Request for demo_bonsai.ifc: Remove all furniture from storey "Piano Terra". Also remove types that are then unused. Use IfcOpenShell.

First a look at what the model holds.

```python
import ifcopenshell
import ifcopenshell.util.element

model = ifcopenshell.open("demo_bonsai.ifc")
print(model.schema)
storey = next(s for s in model.by_type("IfcBuildingStorey") if s.Name == "Piano Terra")
furniture = [e for e in ifcopenshell.util.element.get_decomposition(storey) if e.is_a("IfcFurnishingElement")]
seen = {}
for e in furniture:
    element_type = ifcopenshell.util.element.get_type(e)
    name = element_type.Name if element_type not in (None, e) else None
    seen[name] = seen.get(name, 0) + 1
for name, count in sorted(seen.items(), key=str):
    print(count, "x", name)
```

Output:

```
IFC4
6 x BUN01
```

```python
import ifcopenshell
import ifcopenshell.api.root
import ifcopenshell.util.element

model = ifcopenshell.open("demo_bonsai.ifc")

storey = next(s for s in model.by_type("IfcBuildingStorey") if s.Name == "Piano Terra")
furniture = [e for e in ifcopenshell.util.element.get_decomposition(storey) if e.is_a("IfcFurnishingElement")]
types = {ifcopenshell.util.element.get_type(e) for e in furniture} - {None, *furniture}

for e in furniture:
    ifcopenshell.api.root.remove_product(model, product=e)
print(len(furniture), "removed")

unused = [t for t in types if not ifcopenshell.util.element.get_types(t)]
for t in unused:
    ifcopenshell.api.root.remove_product(model, product=t)
print(len(unused), "unused types removed")

model.write("demo_bonsai_edited.ifc")
```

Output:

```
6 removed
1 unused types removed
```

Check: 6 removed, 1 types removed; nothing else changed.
